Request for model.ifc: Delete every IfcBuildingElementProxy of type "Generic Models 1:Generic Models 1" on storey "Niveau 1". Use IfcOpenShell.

First a look at what the model holds.

```python
import ifcopenshell
import ifcopenshell.util.element

model = ifcopenshell.open("model.ifc")
print(model.schema)
storey = next(s for s in model.by_type("IfcBuildingStorey") if s.Name == "Niveau 1")
proxies = [e for e in ifcopenshell.util.element.get_decomposition(storey) if e.is_a("IfcBuildingElementProxy")]
seen = {}
for e in proxies:
    element_type = ifcopenshell.util.element.get_type(e)
    name = element_type.Name if element_type not in (None, e) else None
    seen[name] = seen.get(name, 0) + 1
for name, count in sorted(seen.items(), key=str):
    print(count, "x", name)
```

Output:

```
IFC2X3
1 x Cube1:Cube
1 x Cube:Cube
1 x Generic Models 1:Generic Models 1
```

```python
import ifcopenshell
import ifcopenshell.api.root
import ifcopenshell.util.element

model = ifcopenshell.open("model.ifc")

storey = next(s for s in model.by_type("IfcBuildingStorey") if s.Name == "Niveau 1")
proxies = [e for e in ifcopenshell.util.element.get_decomposition(storey) if e.is_a("IfcBuildingElementProxy")]
targets = [e for e in proxies if (t := ifcopenshell.util.element.get_type(e)) not in (None, e) and t.Name == "Generic Models 1:Generic Models 1"]

for e in targets:
    ifcopenshell.api.root.remove_product(model, product=e)
print(len(targets), "removed")

model.write("model_edited.ifc")
```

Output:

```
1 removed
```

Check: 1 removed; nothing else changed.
